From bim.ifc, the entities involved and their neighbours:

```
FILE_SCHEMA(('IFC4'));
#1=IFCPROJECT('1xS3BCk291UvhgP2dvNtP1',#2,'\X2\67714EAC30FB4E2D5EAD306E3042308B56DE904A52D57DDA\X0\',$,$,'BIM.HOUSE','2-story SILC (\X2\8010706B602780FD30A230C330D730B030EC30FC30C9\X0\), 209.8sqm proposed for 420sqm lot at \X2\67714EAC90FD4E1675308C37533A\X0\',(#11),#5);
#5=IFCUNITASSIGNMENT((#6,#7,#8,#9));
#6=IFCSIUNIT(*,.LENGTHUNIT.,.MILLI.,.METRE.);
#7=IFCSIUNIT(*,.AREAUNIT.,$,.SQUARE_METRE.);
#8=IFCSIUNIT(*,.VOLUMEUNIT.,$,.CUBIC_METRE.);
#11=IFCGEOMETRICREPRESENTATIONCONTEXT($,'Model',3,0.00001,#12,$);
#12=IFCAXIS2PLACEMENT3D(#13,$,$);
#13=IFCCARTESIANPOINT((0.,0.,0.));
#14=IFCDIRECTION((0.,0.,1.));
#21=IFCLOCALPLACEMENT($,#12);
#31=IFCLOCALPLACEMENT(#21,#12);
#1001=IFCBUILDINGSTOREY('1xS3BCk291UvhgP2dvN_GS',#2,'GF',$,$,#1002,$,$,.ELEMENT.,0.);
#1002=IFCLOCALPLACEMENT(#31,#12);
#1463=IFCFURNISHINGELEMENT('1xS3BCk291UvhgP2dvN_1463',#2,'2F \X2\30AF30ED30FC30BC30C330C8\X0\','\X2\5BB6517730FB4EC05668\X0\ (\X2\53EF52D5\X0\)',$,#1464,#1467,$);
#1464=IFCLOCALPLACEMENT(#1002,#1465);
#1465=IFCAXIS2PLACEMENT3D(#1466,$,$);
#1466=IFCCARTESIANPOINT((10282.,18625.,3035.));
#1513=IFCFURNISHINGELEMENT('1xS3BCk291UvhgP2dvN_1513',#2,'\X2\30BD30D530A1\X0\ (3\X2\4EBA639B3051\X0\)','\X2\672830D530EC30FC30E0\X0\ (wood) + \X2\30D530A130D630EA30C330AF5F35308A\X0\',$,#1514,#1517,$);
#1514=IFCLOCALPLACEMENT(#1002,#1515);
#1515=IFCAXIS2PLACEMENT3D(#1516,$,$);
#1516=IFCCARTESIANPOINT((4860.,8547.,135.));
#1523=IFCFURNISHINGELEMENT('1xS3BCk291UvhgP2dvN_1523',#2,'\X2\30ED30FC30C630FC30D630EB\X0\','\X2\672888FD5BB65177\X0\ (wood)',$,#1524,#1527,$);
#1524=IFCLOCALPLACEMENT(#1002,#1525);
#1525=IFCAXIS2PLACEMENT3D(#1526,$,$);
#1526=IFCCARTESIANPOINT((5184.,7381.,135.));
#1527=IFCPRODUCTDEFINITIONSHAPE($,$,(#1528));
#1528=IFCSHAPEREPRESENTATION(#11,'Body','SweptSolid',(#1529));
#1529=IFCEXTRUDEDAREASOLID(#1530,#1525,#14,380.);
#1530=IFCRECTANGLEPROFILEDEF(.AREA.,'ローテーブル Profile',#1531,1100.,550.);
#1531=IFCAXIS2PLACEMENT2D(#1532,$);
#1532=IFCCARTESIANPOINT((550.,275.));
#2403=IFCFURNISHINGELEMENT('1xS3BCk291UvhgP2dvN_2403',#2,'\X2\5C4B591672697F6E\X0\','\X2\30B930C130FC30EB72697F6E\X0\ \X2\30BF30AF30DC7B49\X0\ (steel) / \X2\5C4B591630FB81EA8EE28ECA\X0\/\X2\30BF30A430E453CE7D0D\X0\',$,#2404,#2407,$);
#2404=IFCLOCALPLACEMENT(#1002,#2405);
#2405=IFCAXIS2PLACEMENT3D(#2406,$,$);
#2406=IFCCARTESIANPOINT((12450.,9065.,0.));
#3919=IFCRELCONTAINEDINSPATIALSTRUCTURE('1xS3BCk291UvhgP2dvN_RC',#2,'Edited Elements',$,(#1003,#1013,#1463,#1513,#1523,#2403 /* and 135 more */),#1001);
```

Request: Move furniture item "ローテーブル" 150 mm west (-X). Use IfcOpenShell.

```python
import ifcopenshell
import ifcopenshell.api.geometry
import ifcopenshell.util.placement
import ifcopenshell.util.unit

model = ifcopenshell.open("bim.ifc")
unit_scale = ifcopenshell.util.unit.calculate_unit_scale(model)

item = model.by_id(1523)
matrix = ifcopenshell.util.placement.get_local_placement(item.ObjectPlacement)
matrix[0, 3] -= 0.15 / unit_scale
ifcopenshell.api.geometry.edit_object_placement(model, product=item, matrix=matrix, is_si=False)

print(ifcopenshell.util.placement.get_local_placement(item.ObjectPlacement).round(3) + 0.0)

model.write("bim_rev.ifc")
```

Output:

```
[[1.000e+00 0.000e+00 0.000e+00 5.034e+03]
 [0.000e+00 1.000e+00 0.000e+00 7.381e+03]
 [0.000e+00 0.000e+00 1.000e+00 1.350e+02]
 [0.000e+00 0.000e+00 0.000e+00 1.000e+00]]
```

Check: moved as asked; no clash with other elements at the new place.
